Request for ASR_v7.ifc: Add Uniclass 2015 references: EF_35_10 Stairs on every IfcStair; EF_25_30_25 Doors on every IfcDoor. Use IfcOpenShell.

First a look at what the model holds.

```python
import ifcopenshell

model = ifcopenshell.open("ASR_v7.ifc")
print(model.schema)
print("classifications:", [c.Name for c in model.by_type("IfcClassification")])
for ifc_class in ("IfcDoor", "IfcRoof", "IfcStair", "IfcWall", "IfcWindow"):
    print(ifc_class, len(model.by_type(ifc_class)))
```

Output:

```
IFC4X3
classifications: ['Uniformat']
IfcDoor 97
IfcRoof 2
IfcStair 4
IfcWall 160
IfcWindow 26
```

```python
import ifcopenshell
import ifcopenshell.api.classification

model = ifcopenshell.open("ASR_v7.ifc")

system = ifcopenshell.api.classification.add_classification(model, classification="Uniclass 2015")

codes = {
    "IfcStair": ("EF_35_10", "Stairs"),
    "IfcDoor": ("EF_25_30_25", "Doors"),
}
for ifc_class, (code, name) in codes.items():
    products = model.by_type(ifc_class)
    ifcopenshell.api.classification.add_reference(
        model, products=products, classification=system, identification=code, name=name
    )
    print(code, len(products))

model.write("ASR_v7_edited.ifc")
```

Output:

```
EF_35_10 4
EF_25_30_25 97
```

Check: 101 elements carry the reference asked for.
